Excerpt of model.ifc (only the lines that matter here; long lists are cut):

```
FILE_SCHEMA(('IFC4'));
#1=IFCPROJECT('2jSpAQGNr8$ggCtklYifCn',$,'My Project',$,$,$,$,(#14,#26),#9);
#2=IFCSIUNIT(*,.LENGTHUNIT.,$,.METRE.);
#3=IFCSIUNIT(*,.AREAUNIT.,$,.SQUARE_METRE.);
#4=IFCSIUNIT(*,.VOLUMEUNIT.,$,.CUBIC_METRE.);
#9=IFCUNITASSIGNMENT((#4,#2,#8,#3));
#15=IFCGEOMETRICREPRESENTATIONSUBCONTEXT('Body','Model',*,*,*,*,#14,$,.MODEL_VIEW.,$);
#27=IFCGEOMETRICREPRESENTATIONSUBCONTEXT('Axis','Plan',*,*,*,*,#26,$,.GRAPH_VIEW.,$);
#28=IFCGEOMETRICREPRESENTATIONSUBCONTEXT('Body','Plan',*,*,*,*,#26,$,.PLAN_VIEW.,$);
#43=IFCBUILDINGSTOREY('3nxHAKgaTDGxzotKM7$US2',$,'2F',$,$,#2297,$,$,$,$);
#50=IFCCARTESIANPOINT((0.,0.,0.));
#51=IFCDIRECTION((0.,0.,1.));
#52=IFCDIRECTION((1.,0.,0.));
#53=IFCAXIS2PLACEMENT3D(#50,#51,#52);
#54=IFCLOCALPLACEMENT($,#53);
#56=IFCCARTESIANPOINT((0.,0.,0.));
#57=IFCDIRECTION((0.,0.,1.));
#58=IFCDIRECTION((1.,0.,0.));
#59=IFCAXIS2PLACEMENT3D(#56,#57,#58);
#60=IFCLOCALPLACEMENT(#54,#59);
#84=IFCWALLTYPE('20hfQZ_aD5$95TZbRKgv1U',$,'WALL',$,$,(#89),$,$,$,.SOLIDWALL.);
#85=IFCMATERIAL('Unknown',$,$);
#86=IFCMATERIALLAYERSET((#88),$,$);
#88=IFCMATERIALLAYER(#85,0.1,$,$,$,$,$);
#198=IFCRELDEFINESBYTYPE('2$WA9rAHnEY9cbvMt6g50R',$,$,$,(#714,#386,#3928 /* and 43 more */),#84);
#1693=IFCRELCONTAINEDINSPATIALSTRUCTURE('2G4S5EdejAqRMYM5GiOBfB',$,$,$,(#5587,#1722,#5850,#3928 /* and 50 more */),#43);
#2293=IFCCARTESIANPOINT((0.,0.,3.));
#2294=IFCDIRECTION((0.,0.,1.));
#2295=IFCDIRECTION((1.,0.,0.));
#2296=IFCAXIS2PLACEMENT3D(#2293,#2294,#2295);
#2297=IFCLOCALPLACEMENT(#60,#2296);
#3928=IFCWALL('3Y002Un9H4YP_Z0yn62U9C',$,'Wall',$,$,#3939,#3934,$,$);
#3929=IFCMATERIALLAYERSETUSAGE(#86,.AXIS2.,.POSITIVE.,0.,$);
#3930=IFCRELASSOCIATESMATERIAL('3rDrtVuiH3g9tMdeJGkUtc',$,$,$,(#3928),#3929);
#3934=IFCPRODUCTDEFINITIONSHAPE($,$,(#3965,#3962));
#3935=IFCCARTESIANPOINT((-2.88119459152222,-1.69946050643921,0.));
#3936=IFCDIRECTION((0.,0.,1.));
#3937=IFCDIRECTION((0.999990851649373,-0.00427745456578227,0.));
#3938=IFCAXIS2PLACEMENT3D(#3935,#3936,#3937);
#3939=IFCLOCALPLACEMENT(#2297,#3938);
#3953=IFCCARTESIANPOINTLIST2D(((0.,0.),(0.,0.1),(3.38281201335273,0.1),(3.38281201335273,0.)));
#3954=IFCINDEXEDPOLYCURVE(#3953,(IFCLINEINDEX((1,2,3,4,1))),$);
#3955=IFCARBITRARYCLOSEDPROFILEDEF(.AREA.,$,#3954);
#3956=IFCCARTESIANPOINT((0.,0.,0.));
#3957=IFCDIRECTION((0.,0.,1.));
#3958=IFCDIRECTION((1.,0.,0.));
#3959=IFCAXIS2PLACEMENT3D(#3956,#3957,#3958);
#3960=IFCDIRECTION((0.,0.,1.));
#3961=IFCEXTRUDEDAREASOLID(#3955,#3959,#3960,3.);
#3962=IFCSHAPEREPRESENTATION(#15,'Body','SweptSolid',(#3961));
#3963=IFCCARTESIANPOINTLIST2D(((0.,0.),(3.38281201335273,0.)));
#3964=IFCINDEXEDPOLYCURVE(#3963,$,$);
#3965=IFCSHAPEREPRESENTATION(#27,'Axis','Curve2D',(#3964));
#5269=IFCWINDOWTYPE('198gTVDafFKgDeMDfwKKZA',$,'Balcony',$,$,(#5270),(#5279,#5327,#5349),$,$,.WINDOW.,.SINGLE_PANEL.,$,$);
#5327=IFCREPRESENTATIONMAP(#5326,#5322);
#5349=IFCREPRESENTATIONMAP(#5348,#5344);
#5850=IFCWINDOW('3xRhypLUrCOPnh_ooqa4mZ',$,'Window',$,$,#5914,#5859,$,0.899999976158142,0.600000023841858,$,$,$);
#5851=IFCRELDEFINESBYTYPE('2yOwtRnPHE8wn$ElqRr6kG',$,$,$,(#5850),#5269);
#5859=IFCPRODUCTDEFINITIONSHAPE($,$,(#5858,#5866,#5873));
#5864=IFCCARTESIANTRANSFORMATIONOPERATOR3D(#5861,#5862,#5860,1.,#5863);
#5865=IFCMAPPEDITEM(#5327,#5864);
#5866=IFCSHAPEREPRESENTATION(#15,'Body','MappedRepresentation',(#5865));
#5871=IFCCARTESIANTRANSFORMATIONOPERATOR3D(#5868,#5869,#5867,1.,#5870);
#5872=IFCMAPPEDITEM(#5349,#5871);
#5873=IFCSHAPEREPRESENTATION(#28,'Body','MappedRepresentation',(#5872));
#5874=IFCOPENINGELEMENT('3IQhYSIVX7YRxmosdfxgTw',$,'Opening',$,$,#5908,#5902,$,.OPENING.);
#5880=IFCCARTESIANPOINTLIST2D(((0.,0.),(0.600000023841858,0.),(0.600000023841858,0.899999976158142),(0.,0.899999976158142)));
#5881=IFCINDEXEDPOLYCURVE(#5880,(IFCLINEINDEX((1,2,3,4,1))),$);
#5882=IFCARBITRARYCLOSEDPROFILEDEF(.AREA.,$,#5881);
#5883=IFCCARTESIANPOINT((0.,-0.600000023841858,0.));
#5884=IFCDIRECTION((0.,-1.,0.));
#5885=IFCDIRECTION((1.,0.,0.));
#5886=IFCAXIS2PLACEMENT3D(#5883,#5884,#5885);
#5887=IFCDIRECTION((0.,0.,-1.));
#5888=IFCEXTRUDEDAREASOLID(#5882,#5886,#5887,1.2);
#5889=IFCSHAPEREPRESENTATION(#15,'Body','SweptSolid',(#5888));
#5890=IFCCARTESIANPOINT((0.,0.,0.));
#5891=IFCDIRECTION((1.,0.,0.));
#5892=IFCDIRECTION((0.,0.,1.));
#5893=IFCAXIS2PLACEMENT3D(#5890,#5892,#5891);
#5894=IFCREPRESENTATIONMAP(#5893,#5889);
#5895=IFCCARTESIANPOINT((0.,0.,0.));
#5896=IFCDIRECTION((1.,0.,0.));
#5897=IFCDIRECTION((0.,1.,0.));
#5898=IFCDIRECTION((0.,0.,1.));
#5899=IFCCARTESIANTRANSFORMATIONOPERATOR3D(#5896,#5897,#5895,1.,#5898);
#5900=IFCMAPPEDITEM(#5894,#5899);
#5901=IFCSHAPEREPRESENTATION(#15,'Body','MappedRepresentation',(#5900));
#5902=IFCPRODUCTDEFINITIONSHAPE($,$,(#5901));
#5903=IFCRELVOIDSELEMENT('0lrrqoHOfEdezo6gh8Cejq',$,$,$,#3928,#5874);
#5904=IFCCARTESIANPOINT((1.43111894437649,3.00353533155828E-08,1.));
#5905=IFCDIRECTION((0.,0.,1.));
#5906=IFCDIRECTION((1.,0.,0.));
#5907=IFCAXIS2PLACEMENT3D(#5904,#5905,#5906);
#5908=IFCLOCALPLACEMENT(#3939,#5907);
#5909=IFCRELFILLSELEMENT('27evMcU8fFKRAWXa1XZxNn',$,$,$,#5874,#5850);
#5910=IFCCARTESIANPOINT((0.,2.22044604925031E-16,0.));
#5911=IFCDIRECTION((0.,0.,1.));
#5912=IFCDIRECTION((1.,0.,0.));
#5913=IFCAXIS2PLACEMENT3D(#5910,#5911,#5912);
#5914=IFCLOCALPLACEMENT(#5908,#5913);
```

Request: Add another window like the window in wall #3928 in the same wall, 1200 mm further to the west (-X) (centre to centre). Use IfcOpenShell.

```python
import ifcopenshell
import ifcopenshell.api.feature
import ifcopenshell.api.geometry
import ifcopenshell.api.root
import ifcopenshell.geom
import ifcopenshell.util.element
import ifcopenshell.util.placement
import ifcopenshell.util.shape
import ifcopenshell.util.unit

model = ifcopenshell.open("model.ifc")
unit_scale = ifcopenshell.util.unit.calculate_unit_scale(model)
settings = ifcopenshell.geom.settings()


def volume(element):
    """Net volume in cubic metres, openings subtracted."""
    shape = ifcopenshell.geom.create_shape(settings, element)
    return ifcopenshell.util.shape.get_volume(shape.geometry)


window = model.by_guid("3xRhypLUrCOPnh_ooqa4mZ")
opening = window.FillsVoids[0].RelatingOpeningElement
wall = opening.VoidsElements[0].RelatingBuildingElement
before = volume(wall)
shift = ifcopenshell.util.placement.get_local_placement(wall.ObjectPlacement)[:3, 0] * -1.2 / unit_scale

# copy_class copies the void relationship, type, container and properties, but no geometry.
new_opening = ifcopenshell.api.root.copy_class(model, product=opening)
new_opening.Representation = ifcopenshell.util.element.copy_deep(
    model, opening.Representation, exclude=["IfcGeometricRepresentationContext", "IfcRepresentationMap"]
)
new_window = ifcopenshell.api.root.copy_class(model, product=window)
new_window.Representation = ifcopenshell.util.element.copy_deep(
    model, window.Representation, exclude=["IfcGeometricRepresentationContext", "IfcRepresentationMap"]
)
ifcopenshell.api.feature.add_filling(model, opening=new_opening, element=new_window)

for old, new in ((opening, new_opening), (window, new_window)):
    matrix = ifcopenshell.util.placement.get_local_placement(old.ObjectPlacement)
    matrix[:3, 3] += shift
    ifcopenshell.api.geometry.edit_object_placement(model, product=new, matrix=matrix, is_si=False)

after = volume(wall)

print(f"wall volume {before:.3f} -> {after:.3f} m3")

model.write("model_edited.ifc")
```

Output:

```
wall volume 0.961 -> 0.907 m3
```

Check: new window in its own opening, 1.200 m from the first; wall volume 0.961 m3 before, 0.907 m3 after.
